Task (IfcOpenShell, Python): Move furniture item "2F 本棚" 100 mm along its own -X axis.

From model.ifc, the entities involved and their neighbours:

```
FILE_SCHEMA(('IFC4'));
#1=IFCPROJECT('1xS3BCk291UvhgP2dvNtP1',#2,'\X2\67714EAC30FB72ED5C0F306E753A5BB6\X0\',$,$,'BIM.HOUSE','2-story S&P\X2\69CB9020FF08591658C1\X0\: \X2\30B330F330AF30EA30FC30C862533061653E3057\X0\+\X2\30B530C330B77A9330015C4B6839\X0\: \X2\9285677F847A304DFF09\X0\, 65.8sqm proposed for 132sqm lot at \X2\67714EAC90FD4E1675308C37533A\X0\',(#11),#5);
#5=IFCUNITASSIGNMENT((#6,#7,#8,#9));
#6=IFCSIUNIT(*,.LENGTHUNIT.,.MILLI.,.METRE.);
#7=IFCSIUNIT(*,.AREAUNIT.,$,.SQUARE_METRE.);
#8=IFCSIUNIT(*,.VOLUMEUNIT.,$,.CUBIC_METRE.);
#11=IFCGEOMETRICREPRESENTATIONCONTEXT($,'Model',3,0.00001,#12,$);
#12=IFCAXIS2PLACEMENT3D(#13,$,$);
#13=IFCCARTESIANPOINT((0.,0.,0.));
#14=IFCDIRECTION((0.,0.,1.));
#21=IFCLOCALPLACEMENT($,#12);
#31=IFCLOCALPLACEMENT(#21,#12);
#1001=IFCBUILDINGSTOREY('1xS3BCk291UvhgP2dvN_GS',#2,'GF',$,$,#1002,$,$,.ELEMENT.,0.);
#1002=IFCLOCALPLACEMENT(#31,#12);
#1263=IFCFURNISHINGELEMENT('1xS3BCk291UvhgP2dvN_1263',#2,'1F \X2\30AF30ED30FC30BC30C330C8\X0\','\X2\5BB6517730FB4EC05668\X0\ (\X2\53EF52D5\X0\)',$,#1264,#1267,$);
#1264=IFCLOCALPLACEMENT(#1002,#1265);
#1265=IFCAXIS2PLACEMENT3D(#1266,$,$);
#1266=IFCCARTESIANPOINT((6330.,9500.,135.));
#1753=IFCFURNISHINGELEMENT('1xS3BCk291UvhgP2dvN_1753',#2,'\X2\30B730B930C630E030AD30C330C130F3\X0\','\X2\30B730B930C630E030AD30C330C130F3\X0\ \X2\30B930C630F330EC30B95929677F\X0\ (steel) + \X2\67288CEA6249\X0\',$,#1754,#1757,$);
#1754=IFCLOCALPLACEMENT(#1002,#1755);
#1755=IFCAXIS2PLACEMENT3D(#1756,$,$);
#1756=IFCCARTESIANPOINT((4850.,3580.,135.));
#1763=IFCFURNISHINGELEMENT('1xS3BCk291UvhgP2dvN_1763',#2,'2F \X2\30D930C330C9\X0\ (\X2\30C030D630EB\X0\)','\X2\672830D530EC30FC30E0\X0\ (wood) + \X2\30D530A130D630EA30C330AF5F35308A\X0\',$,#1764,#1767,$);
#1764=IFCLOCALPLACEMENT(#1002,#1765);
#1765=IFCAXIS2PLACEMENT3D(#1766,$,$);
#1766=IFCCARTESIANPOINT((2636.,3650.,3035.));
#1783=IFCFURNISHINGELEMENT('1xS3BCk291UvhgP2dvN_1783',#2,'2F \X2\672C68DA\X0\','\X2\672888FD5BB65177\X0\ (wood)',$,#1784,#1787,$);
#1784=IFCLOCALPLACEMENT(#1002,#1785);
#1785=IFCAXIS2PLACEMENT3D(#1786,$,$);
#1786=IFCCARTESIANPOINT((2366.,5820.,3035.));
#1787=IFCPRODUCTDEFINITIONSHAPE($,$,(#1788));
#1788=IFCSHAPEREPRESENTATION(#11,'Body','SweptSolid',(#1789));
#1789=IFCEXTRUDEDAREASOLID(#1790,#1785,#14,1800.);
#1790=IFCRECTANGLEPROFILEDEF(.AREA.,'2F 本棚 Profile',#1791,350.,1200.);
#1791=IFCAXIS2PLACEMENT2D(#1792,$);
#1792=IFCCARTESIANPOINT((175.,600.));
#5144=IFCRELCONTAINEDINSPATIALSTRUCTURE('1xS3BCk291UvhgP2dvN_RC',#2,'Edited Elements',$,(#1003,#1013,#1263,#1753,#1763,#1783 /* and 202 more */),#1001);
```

```python
import ifcopenshell
import ifcopenshell.api.geometry
import ifcopenshell.util.placement
import ifcopenshell.util.unit

model = ifcopenshell.open("model.ifc")
unit_scale = ifcopenshell.util.unit.calculate_unit_scale(model)

item = model.by_guid("1xS3BCk291UvhgP2dvN_1783")
matrix = ifcopenshell.util.placement.get_local_placement(item.ObjectPlacement)
matrix[:3, 3] -= matrix[:3, 0] * 0.1 / unit_scale
ifcopenshell.api.geometry.edit_object_placement(model, product=item, matrix=matrix, is_si=False)

print(ifcopenshell.util.placement.get_local_placement(item.ObjectPlacement).round(3) + 0.0)

model.write("model_updated.ifc")
```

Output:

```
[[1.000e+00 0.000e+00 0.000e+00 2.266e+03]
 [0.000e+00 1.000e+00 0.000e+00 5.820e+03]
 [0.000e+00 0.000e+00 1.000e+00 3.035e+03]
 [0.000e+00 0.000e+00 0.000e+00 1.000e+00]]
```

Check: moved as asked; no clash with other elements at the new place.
